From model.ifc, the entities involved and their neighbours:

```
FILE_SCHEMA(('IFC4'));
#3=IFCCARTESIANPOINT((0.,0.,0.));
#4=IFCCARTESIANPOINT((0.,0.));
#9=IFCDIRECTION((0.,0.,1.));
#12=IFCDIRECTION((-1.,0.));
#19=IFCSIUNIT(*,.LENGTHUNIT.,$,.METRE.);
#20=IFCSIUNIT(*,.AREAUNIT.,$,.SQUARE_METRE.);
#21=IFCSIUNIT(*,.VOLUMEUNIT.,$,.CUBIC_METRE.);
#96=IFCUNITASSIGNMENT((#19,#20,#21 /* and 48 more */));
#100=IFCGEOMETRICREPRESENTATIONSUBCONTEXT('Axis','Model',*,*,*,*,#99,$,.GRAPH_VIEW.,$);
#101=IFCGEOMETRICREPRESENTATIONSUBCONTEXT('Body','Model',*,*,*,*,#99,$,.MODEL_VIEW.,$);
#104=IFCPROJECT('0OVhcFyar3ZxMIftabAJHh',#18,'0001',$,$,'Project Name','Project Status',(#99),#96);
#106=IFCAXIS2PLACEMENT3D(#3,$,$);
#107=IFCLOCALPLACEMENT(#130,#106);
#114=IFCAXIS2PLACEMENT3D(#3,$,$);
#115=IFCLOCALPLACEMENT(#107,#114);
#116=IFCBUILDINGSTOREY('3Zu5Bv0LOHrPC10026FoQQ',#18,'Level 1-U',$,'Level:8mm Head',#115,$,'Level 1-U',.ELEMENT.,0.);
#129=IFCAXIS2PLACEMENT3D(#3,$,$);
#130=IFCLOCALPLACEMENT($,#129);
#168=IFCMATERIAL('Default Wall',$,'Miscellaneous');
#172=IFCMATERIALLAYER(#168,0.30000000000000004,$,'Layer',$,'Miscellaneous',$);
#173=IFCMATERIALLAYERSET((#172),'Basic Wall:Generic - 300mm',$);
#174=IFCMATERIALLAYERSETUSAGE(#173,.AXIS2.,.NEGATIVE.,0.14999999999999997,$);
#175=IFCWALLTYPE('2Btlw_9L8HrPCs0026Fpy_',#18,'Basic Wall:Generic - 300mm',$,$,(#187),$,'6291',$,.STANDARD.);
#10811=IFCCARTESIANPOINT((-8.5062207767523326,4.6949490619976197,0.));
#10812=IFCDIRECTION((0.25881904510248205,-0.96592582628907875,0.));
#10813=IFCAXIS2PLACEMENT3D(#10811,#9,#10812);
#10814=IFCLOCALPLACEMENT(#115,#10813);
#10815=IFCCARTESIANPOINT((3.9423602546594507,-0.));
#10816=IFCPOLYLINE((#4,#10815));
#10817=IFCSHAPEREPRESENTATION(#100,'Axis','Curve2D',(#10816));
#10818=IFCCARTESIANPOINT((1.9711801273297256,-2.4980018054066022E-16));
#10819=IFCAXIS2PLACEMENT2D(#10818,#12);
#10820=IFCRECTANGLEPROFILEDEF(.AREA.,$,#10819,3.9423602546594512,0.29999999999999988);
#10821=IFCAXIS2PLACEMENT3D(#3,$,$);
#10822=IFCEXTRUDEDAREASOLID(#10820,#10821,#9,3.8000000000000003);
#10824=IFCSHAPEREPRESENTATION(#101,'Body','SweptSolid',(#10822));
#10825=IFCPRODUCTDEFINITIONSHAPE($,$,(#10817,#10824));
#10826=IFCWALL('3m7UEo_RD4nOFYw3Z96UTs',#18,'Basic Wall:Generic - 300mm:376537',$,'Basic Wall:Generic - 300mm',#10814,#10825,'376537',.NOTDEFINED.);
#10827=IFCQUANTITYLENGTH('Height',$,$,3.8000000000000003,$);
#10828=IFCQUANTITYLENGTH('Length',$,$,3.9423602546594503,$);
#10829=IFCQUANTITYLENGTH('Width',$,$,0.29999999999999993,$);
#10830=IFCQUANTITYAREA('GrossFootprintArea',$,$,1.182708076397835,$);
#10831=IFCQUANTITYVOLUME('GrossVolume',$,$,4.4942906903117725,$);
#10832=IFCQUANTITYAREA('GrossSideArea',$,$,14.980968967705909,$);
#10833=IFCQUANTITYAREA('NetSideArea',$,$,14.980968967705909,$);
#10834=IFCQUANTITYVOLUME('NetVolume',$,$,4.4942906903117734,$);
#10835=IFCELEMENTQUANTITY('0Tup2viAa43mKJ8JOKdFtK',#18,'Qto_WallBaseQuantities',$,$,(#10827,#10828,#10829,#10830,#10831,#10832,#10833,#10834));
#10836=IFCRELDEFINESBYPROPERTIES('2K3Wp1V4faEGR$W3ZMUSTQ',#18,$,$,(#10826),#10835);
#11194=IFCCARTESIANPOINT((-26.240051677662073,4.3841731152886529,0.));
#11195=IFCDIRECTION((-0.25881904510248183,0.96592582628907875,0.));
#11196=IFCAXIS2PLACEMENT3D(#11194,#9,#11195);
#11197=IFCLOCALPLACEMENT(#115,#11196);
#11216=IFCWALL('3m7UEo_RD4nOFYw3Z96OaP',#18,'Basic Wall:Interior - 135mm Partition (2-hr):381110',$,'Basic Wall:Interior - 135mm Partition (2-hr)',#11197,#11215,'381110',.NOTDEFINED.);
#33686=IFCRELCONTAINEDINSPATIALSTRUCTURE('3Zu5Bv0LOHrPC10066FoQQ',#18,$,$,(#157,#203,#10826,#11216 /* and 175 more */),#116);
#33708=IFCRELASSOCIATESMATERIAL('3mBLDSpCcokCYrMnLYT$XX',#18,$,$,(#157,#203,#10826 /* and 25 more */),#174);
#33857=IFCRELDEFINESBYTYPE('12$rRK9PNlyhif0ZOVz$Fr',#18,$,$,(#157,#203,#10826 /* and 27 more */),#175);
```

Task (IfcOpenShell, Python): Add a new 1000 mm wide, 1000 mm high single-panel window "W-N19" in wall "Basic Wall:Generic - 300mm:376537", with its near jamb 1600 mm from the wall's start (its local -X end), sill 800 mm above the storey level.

```python
import numpy as np
import ifcopenshell
import ifcopenshell.api.feature
import ifcopenshell.api.geometry
import ifcopenshell.api.pset
import ifcopenshell.api.root
import ifcopenshell.api.spatial
import ifcopenshell.geom
import ifcopenshell.util.element
import ifcopenshell.util.placement
import ifcopenshell.util.representation
import ifcopenshell.util.shape
import ifcopenshell.util.unit

model = ifcopenshell.open("model.ifc")
unit_scale = ifcopenshell.util.unit.calculate_unit_scale(model)
area_scale = ifcopenshell.util.unit.calculate_unit_scale(model, "AREAUNIT")
volume_scale = ifcopenshell.util.unit.calculate_unit_scale(model, "VOLUMEUNIT")
settings = ifcopenshell.geom.settings()


def volume(element):
    """Net volume in cubic metres, openings subtracted."""
    shape = ifcopenshell.geom.create_shape(settings, element)
    return ifcopenshell.util.shape.get_volume(shape.geometry)


wall = model.by_guid("3m7UEo_RD4nOFYw3Z96UTs")
storey = ifcopenshell.util.element.get_container(wall, ifc_class="IfcBuildingStorey")
context = ifcopenshell.util.representation.get_context(model, "Model", "Body", "MODEL_VIEW")
before = volume(wall)

width, height, from_end, sill = 1, 1, 1.6, 0.8  # metres

# The wall runs along its own X axis, and the end named is its -X end.
wall_shape = ifcopenshell.geom.create_shape(settings, wall)
x, y, z = ifcopenshell.util.shape.get_vertices(wall_shape.geometry).T
start = x.min() + from_end
face, thickness = float(y.min()), float(y.max() - y.min())
wall_matrix = ifcopenshell.util.placement.get_local_placement(wall.ObjectPlacement)
level = ifcopenshell.util.placement.get_local_placement(storey.ObjectPlacement)[2, 3]


def in_wall(x, y):
    """Placement at x, y metres in the wall's axes, at sill height."""
    matrix = wall_matrix.copy()
    matrix[:, 3] = wall_matrix @ np.array([x / unit_scale, y / unit_scale, 0.0, 1.0])
    matrix[2, 3] = level + sill / unit_scale
    return matrix


# Opening: a box that overshoots both wall faces by 50 mm.
opening = ifcopenshell.api.root.create_entity(model, ifc_class="IfcOpeningElement", predefined_type="OPENING")
box = ifcopenshell.api.geometry.add_wall_representation(
    model, context=context, length=width, height=height, thickness=thickness + 0.1
)
ifcopenshell.api.geometry.assign_representation(model, product=opening, representation=box)
ifcopenshell.api.geometry.edit_object_placement(model, product=opening, matrix=in_wall(start, face - 0.05), is_si=False)
ifcopenshell.api.feature.add_feature(model, feature=opening, element=wall)

window = ifcopenshell.api.root.create_entity(model, ifc_class="IfcWindow", name="W-N19", predefined_type="WINDOW")
window.OverallWidth, window.OverallHeight = width / unit_scale, height / unit_scale
window.PartitioningType = "SINGLE_PANEL"
body = ifcopenshell.api.geometry.add_window_representation(
    model,
    context=context,
    overall_width=window.OverallWidth,
    overall_height=window.OverallHeight,
    partition_type="SINGLE_PANEL",
)
ifcopenshell.api.geometry.assign_representation(model, product=window, representation=body)
ifcopenshell.api.spatial.assign_container(model, products=[window], relating_structure=storey)
ifcopenshell.api.feature.add_filling(model, opening=opening, element=window)

# Centre the window in the wall's thickness.
ifcopenshell.api.geometry.edit_object_placement(model, product=window, matrix=in_wall(start, face), is_si=False)
window_shape = ifcopenshell.geom.create_shape(settings, window)
depth = ifcopenshell.util.shape.get_vertices(window_shape.geometry)[:, 1]
offset = face + thickness / 2 - (depth.min() + depth.max()) / 2
ifcopenshell.api.geometry.edit_object_placement(model, product=window, matrix=in_wall(start, offset), is_si=False)

after = volume(wall)

# Update the wall's stored quantities.
qto = model.by_id(ifcopenshell.util.element.get_pset(wall, "Qto_WallBaseQuantities", should_inherit=False)["id"])
ifcopenshell.api.pset.edit_qto(model, qto=qto, properties={
    "NetSideArea": after / thickness / area_scale,
    "NetVolume": after / volume_scale,
})

print(f"wall volume {before:.3f} -> {after:.3f} m3")

model.write("model_v2.ifc")
```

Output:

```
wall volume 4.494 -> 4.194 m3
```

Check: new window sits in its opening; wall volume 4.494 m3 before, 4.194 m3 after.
